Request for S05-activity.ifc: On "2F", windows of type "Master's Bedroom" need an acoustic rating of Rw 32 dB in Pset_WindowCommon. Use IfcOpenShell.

First a look at what the model holds.

```python
import ifcopenshell
import ifcopenshell.util.element

model = ifcopenshell.open("S05-activity.ifc")
print(model.schema)
storey = next(s for s in model.by_type("IfcBuildingStorey") if s.Name == "2F")
windows = [e for e in ifcopenshell.util.element.get_decomposition(storey) if e.is_a("IfcWindow")]
seen = {}
for e in windows:
    element_type = ifcopenshell.util.element.get_type(e)
    key = (element_type.Name if element_type != e and element_type else None, ifcopenshell.util.element.get_pset(e, "Pset_WindowCommon", "AcousticRating"))
    seen[key] = seen.get(key, 0) + 1
for (name, value), count in sorted(seen.items(), key=str):
    print(count, "x", name, "|", value)
```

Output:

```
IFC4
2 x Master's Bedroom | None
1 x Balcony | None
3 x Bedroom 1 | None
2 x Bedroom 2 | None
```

```python
import ifcopenshell
import ifcopenshell.api.pset
import ifcopenshell.util.element

model = ifcopenshell.open("S05-activity.ifc")

storey = next(s for s in model.by_type("IfcBuildingStorey") if s.Name == "2F")
windows = [e for e in ifcopenshell.util.element.get_decomposition(storey) if e.is_a("IfcWindow")]

count = 0
for e in windows:
    element_type = ifcopenshell.util.element.get_type(e)
    if element_type in (None, e) or element_type.Name != "Master's Bedroom":
        continue
    # add_pset returns the element's existing set when there is one.
    pset = ifcopenshell.api.pset.add_pset(model, product=e, name="Pset_WindowCommon")
    ifcopenshell.api.pset.edit_pset(model, pset=pset, properties={"AcousticRating": "Rw 32 dB"})
    count += 1

print(count, "windows updated")

model.write("S05-activity_updated.ifc")
```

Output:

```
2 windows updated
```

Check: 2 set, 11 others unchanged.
